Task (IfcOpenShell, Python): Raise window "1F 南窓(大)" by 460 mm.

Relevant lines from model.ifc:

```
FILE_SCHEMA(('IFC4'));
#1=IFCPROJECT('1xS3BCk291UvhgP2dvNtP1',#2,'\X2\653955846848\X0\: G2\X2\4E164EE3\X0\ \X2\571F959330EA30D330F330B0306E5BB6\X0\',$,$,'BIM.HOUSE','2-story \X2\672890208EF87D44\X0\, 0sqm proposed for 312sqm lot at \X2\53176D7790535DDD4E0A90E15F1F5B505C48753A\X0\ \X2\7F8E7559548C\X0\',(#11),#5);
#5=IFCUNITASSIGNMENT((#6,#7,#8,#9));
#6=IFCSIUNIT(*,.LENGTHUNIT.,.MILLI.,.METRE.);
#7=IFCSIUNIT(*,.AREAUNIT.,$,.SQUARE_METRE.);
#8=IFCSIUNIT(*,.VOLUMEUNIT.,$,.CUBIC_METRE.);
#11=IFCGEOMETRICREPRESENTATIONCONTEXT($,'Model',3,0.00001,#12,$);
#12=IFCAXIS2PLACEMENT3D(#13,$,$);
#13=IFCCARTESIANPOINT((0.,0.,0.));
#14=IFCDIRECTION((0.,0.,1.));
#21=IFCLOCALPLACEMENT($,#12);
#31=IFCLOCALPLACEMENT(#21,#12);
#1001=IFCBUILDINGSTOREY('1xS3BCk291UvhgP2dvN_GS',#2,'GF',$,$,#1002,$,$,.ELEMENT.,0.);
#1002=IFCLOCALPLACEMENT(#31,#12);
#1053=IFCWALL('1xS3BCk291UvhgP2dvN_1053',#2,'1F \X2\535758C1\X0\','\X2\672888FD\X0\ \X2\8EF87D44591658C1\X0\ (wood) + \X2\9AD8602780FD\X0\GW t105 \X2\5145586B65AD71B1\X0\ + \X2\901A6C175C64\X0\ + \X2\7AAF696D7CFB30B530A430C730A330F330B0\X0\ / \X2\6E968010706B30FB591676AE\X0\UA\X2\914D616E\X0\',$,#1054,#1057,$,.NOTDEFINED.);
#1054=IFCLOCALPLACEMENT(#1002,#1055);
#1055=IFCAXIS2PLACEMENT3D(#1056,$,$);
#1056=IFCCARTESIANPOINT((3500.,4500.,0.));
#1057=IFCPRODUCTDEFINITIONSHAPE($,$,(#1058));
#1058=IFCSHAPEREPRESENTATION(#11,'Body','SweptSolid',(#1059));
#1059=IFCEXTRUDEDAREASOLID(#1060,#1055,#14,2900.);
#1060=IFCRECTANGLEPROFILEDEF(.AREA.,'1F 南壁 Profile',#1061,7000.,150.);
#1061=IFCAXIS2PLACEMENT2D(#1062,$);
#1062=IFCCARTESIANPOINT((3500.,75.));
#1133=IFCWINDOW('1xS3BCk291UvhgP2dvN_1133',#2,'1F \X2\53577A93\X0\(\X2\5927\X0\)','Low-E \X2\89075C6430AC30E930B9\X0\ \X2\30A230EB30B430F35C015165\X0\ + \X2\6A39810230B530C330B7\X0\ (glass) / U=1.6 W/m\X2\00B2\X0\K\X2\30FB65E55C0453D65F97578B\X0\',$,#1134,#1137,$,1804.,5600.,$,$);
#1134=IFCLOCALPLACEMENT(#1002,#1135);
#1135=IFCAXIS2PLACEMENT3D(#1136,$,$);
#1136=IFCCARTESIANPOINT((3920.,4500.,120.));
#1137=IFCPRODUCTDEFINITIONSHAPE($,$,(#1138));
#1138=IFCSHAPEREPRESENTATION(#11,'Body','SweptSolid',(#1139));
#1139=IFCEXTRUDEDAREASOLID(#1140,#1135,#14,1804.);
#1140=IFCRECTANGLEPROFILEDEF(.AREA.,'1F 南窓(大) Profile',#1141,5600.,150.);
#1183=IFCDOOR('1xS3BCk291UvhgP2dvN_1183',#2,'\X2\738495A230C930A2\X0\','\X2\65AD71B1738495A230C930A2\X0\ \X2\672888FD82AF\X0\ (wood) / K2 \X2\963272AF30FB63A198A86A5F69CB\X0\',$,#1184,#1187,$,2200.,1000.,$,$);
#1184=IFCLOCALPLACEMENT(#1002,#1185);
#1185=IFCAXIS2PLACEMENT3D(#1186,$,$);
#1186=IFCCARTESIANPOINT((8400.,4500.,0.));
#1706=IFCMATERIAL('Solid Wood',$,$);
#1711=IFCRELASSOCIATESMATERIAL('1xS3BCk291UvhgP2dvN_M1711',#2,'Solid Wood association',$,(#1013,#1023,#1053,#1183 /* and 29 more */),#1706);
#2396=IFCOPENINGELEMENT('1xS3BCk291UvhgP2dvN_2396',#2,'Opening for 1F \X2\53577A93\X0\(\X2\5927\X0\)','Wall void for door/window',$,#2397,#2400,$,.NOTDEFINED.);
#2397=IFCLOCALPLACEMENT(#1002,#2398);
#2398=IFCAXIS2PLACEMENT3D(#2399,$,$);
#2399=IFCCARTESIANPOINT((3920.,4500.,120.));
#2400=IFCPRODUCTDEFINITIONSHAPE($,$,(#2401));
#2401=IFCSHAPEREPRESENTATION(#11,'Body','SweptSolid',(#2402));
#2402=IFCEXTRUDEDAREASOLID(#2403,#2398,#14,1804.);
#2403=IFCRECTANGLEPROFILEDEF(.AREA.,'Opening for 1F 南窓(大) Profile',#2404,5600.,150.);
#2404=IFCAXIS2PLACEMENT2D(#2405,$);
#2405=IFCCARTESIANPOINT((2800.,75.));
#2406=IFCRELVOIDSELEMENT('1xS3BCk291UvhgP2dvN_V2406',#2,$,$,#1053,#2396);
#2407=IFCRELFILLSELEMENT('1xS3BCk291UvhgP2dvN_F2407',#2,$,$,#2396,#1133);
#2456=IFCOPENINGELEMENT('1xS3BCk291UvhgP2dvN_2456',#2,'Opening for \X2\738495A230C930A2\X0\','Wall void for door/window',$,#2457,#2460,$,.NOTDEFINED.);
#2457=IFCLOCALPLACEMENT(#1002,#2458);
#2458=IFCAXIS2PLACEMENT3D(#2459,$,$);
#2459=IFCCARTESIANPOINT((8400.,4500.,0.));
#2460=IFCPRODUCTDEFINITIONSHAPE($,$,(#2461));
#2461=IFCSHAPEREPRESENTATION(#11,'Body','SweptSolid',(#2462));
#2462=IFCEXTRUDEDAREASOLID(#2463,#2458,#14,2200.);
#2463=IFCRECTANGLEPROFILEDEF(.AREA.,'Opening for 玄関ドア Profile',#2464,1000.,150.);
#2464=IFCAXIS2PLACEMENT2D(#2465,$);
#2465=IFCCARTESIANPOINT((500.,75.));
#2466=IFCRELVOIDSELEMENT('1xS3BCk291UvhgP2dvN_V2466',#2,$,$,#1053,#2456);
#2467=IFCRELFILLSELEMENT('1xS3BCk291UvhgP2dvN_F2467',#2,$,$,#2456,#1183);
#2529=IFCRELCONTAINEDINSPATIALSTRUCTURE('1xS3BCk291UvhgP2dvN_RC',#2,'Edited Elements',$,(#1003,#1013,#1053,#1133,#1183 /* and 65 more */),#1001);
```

```python
import numpy as np
import ifcopenshell
import ifcopenshell.api.geometry
import ifcopenshell.util.placement
import ifcopenshell.util.unit

model = ifcopenshell.open("model.ifc")
unit_scale = ifcopenshell.util.unit.calculate_unit_scale(model)

window = model.by_id(1133)
opening = window.FillsVoids[0].RelatingOpeningElement
dz = 460.0

shift = np.array([0.0, 0.0, dz])
# The window is not placed relative to its opening, so move both.
for product in (opening, window):
    matrix = ifcopenshell.util.placement.get_local_placement(product.ObjectPlacement)
    matrix[:3, 3] += shift
    ifcopenshell.api.geometry.edit_object_placement(model, product=product, matrix=matrix, is_si=False)

print(f"moved by {dz * unit_scale:+.3f} m")

model.write("model_rev.ifc")
```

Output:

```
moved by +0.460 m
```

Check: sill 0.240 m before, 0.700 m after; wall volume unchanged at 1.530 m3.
